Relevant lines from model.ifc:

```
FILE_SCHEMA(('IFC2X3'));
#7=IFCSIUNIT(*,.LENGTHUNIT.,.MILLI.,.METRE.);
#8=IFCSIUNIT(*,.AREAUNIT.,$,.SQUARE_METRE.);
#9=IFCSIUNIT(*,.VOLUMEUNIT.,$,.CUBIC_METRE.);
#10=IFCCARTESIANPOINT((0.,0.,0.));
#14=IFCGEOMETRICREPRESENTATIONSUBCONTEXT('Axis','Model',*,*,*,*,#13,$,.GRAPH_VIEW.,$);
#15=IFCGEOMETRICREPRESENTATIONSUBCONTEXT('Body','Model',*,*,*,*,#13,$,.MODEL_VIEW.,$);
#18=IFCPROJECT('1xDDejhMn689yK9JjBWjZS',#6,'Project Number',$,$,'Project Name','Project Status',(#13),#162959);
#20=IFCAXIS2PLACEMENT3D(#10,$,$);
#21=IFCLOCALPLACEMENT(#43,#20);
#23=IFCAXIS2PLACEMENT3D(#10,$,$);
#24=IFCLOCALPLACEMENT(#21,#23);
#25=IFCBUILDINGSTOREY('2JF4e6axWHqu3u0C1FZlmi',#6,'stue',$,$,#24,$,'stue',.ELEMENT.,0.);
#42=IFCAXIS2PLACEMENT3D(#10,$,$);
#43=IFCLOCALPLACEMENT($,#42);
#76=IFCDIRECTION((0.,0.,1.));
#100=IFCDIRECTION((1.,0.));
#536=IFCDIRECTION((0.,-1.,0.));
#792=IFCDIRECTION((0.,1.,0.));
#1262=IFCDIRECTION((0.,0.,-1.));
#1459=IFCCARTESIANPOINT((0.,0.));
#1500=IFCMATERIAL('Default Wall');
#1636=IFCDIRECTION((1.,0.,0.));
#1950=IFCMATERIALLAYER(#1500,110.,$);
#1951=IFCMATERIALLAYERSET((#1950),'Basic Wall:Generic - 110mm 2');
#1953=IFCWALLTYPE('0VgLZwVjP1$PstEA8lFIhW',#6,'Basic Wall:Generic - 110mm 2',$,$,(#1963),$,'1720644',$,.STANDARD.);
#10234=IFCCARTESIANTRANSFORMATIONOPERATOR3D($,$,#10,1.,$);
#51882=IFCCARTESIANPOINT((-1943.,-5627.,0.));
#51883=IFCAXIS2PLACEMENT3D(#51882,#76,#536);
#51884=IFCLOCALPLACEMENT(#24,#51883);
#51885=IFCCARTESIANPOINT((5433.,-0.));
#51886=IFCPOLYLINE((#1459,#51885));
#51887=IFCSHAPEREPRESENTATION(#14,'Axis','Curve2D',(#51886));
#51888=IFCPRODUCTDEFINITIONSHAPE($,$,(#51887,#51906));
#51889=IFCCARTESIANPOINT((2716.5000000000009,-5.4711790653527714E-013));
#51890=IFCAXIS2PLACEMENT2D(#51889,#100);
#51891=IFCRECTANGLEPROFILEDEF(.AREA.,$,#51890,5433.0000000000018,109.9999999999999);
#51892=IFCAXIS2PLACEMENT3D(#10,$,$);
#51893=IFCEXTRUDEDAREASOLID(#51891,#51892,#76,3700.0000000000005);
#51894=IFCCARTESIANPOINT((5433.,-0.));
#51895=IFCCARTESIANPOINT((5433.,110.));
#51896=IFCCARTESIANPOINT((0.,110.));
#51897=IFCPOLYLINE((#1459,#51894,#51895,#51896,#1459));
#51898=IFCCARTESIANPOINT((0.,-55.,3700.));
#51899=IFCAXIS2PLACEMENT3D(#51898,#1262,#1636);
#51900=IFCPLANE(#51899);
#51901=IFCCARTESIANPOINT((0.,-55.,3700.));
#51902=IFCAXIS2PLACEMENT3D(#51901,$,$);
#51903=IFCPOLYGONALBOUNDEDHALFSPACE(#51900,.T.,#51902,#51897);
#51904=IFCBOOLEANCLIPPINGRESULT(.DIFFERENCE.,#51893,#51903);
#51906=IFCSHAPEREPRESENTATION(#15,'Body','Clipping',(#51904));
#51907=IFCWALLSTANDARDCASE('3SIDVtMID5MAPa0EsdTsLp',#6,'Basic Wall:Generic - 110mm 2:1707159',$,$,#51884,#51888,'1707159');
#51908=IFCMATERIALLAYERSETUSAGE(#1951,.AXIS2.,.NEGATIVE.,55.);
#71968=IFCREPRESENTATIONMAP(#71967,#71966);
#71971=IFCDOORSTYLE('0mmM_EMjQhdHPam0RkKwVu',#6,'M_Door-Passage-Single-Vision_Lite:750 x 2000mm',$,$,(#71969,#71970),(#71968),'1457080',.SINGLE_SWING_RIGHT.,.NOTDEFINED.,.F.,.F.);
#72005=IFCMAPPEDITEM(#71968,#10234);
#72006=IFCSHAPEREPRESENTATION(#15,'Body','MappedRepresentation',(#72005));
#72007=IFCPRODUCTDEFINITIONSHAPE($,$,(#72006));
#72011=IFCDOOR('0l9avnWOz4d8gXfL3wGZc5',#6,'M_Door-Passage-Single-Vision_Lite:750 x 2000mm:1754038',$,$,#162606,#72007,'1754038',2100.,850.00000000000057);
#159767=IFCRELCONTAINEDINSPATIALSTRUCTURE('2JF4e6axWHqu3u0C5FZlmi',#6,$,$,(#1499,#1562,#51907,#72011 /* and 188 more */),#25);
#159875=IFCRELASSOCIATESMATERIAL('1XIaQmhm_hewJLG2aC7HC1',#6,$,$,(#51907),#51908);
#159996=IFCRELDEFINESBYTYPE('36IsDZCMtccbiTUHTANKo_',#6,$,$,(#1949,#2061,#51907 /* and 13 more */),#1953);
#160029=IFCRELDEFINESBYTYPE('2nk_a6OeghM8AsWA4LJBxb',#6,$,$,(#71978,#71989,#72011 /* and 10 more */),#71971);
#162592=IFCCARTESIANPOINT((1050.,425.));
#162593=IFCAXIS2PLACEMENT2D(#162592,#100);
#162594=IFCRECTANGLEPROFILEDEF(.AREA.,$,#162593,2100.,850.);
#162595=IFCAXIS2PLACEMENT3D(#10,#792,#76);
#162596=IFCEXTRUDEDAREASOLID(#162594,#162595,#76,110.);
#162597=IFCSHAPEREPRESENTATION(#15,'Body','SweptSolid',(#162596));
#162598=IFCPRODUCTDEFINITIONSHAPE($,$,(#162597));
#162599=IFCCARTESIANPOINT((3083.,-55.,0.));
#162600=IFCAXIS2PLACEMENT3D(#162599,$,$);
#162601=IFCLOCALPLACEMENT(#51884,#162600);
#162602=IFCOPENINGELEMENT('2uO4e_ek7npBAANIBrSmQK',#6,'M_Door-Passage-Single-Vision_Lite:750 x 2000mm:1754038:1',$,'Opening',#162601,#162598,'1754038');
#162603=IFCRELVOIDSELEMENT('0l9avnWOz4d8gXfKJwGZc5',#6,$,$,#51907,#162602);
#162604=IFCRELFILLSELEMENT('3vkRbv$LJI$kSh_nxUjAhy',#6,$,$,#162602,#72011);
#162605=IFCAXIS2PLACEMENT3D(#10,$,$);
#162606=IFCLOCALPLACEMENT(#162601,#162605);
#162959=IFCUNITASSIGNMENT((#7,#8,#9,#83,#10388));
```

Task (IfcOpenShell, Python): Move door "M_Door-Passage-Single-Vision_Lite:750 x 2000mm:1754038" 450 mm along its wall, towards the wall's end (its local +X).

```python
import ifcopenshell
import ifcopenshell.api.geometry
import ifcopenshell.util.placement
import ifcopenshell.util.unit

model = ifcopenshell.open("model.ifc")
unit_scale = ifcopenshell.util.unit.calculate_unit_scale(model)

door = model.by_guid("0l9avnWOz4d8gXfL3wGZc5")
opening = door.FillsVoids[0].RelatingOpeningElement
wall = opening.VoidsElements[0].RelatingBuildingElement

wall_matrix = ifcopenshell.util.placement.get_local_placement(wall.ObjectPlacement)
shift = wall_matrix[:3, 0] * 0.45 / unit_scale
before = ifcopenshell.util.placement.get_local_placement(door.ObjectPlacement)[:3, 3].copy()

# The door is placed relative to its opening, so it follows when the opening moves.
matrix = ifcopenshell.util.placement.get_local_placement(opening.ObjectPlacement)
matrix[:3, 3] += shift
ifcopenshell.api.geometry.edit_object_placement(
    model, product=opening, matrix=matrix, is_si=False, should_transform_children=True
)

after = ifcopenshell.util.placement.get_local_placement(door.ObjectPlacement)[:3, 3]
print("door moved by", (after - before).round(3) + 0.0)

model.write("model_edited.ifc")
```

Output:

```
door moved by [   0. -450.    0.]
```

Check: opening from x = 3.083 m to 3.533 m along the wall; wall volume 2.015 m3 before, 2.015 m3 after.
